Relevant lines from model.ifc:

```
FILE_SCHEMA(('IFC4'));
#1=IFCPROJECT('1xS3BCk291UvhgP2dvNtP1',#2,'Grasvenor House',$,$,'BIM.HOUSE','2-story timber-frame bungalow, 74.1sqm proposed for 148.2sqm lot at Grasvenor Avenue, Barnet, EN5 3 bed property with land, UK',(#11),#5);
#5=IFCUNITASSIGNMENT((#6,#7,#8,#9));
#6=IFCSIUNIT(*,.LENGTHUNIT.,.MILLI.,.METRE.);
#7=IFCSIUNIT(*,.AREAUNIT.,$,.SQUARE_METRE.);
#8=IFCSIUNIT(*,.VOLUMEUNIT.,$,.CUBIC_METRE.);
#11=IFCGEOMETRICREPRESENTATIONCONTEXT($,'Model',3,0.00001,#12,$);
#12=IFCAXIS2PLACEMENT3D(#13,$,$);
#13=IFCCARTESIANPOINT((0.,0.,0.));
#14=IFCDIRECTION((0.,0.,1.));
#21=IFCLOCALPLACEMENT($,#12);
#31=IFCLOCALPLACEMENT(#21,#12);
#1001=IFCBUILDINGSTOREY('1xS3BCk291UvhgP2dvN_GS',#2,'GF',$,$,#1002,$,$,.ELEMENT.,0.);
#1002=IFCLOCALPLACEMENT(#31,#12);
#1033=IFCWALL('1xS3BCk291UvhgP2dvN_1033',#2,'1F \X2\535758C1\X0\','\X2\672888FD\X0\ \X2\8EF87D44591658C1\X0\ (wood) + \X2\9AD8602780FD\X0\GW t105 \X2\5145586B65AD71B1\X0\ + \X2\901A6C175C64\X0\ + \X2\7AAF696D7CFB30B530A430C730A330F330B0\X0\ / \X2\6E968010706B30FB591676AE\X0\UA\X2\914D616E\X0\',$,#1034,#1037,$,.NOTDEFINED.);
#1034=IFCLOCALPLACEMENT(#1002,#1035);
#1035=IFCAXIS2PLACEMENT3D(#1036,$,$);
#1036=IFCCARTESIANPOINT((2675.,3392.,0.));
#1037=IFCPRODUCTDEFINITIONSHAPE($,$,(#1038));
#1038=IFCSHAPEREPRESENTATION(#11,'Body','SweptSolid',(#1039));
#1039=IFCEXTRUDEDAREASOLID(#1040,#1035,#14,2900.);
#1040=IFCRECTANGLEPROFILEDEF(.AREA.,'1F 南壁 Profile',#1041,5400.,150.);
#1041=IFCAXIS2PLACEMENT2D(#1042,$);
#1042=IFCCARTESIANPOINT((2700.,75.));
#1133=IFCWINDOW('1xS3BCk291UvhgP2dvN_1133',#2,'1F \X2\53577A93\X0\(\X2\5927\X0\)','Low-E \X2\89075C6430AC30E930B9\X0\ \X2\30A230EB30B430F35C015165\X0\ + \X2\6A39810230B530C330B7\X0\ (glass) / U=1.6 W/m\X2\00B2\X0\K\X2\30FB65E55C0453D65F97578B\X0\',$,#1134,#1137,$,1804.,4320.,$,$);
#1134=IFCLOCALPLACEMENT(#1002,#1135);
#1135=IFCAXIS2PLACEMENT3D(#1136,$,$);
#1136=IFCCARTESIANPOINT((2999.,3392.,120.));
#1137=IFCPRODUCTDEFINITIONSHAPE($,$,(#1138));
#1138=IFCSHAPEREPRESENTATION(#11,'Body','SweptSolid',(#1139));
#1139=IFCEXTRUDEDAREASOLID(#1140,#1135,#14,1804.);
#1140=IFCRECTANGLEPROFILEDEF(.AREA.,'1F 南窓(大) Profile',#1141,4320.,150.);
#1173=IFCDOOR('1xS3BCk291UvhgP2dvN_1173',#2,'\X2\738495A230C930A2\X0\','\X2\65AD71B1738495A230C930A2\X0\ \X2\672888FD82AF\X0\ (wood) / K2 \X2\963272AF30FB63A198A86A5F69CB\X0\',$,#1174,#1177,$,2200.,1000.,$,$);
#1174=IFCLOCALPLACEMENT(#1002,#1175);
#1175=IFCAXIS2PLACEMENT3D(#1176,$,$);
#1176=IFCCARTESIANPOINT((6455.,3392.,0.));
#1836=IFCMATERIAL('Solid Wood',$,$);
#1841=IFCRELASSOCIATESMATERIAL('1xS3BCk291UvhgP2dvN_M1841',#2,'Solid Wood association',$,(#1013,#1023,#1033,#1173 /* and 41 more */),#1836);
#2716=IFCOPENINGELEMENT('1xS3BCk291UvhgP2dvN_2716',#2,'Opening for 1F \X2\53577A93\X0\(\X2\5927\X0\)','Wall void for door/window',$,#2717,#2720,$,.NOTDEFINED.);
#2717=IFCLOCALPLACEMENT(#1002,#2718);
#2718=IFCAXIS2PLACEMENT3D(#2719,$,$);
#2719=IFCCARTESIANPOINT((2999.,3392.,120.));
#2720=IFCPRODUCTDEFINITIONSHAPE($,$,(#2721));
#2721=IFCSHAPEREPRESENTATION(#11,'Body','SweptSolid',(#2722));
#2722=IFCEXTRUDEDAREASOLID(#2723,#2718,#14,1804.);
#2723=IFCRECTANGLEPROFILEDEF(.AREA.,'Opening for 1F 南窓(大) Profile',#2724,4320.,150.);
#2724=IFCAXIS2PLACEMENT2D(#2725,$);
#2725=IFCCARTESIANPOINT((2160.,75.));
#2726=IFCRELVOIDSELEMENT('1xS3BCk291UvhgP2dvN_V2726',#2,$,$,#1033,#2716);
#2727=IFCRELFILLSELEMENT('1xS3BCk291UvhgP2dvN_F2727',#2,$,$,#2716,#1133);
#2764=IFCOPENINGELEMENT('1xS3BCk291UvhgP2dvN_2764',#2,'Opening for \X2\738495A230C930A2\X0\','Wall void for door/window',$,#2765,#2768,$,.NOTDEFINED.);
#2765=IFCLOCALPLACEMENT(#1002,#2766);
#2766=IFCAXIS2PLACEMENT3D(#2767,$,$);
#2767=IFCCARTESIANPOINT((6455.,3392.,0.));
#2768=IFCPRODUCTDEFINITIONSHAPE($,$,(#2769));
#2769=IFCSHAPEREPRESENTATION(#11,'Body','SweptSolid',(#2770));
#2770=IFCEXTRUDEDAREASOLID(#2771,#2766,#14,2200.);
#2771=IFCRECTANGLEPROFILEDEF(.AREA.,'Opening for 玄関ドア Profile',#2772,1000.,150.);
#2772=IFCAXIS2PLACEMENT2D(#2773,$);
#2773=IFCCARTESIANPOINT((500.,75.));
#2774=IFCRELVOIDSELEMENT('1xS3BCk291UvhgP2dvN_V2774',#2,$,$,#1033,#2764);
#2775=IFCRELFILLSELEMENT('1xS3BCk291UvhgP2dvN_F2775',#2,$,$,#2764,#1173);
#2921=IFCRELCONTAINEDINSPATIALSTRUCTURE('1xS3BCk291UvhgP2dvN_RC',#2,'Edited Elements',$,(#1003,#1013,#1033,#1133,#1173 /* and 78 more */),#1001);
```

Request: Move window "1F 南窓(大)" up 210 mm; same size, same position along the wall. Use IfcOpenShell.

```python
import numpy as np
import ifcopenshell
import ifcopenshell.api.geometry
import ifcopenshell.util.placement
import ifcopenshell.util.unit

model = ifcopenshell.open("model.ifc")
unit_scale = ifcopenshell.util.unit.calculate_unit_scale(model)

window = model.by_guid("1xS3BCk291UvhgP2dvN_1133")
opening = window.FillsVoids[0].RelatingOpeningElement
dz = 0.21 / unit_scale

shift = np.array([0.0, 0.0, dz])
# The window is not placed relative to its opening, so move both.
for product in (opening, window):
    matrix = ifcopenshell.util.placement.get_local_placement(product.ObjectPlacement)
    matrix[:3, 3] += shift
    ifcopenshell.api.geometry.edit_object_placement(model, product=product, matrix=matrix, is_si=False)

print(f"moved by {dz * unit_scale:+.3f} m")

model.write("model_updated.ifc")
```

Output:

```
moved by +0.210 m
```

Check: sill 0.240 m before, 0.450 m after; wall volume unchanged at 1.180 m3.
